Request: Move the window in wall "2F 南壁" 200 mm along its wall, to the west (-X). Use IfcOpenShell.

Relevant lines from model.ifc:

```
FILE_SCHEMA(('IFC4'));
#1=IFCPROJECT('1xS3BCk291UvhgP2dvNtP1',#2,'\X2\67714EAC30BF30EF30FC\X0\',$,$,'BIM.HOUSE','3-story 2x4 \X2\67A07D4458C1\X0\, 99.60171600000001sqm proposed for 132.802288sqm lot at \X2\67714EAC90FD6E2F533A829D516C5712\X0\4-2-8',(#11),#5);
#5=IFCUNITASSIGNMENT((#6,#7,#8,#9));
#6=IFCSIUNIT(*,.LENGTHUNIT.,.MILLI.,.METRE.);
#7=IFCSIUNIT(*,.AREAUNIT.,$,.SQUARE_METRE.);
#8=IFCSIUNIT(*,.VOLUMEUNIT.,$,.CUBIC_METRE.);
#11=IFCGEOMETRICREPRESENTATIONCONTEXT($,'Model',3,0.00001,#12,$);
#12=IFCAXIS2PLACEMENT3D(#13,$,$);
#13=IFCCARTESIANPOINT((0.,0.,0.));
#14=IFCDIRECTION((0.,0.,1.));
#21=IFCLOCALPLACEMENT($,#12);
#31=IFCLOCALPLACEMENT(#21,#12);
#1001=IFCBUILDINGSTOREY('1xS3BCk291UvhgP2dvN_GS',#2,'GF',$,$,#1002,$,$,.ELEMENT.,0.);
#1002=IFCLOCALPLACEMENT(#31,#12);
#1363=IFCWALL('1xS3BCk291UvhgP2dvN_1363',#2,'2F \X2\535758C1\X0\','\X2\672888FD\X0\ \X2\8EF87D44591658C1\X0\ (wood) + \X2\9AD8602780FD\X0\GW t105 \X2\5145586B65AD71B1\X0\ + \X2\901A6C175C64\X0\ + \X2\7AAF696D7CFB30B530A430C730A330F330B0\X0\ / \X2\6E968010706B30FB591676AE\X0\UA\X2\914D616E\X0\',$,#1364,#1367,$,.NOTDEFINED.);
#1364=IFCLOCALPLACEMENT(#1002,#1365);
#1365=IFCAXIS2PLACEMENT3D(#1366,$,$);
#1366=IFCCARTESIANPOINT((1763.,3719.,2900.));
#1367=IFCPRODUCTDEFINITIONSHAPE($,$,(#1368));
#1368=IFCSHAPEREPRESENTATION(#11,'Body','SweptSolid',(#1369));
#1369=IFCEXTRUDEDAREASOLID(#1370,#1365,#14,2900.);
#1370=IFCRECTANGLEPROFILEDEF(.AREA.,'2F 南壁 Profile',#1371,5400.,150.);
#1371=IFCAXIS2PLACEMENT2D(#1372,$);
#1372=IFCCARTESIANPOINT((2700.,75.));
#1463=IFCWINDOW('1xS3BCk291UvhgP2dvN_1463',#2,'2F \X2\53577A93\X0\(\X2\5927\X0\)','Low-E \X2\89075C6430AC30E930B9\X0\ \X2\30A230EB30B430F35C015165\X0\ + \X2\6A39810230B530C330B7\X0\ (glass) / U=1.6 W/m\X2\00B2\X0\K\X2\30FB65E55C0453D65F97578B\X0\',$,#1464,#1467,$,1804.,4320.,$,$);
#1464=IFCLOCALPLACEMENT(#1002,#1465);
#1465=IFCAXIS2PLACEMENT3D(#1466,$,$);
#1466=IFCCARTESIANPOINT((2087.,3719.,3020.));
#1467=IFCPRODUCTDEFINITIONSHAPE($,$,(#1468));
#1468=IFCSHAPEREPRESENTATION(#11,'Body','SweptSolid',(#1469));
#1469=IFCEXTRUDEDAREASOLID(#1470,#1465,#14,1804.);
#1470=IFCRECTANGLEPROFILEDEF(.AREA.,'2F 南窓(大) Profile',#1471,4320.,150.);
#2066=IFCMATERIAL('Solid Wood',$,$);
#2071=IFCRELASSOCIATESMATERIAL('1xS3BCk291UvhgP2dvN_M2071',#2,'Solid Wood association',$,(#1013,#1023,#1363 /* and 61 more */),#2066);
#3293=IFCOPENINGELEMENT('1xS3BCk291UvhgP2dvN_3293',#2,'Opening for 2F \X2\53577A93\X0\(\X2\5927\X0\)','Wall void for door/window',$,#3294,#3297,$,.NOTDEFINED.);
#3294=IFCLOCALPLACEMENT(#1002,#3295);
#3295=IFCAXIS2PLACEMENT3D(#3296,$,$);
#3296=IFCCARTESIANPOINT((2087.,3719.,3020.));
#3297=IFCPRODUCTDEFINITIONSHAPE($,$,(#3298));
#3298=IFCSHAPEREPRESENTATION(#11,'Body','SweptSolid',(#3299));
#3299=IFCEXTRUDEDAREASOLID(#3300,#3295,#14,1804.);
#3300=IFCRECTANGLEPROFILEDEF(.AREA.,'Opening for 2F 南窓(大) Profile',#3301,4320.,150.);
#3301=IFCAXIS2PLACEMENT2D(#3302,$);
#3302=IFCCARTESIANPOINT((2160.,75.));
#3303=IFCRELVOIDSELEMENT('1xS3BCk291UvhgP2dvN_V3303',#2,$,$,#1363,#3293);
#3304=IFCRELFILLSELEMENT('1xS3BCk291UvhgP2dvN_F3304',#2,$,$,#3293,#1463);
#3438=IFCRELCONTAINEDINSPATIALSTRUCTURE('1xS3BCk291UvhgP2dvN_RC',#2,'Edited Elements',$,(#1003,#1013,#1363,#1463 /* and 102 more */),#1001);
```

```python
import ifcopenshell
import ifcopenshell.api.geometry
import ifcopenshell.util.placement

model = ifcopenshell.open("model.ifc")

window = model.by_guid("1xS3BCk291UvhgP2dvN_1463")
opening = window.FillsVoids[0].RelatingOpeningElement
wall = opening.VoidsElements[0].RelatingBuildingElement

wall_matrix = ifcopenshell.util.placement.get_local_placement(wall.ObjectPlacement)
shift = wall_matrix[:3, 0] * -200.0
before = ifcopenshell.util.placement.get_local_placement(window.ObjectPlacement)[:3, 3].copy()

# The window is not placed relative to its opening, so move both.
for product in (opening, window):
    matrix = ifcopenshell.util.placement.get_local_placement(product.ObjectPlacement)
    matrix[:3, 3] += shift
    ifcopenshell.api.geometry.edit_object_placement(model, product=product, matrix=matrix, is_si=False)

after = ifcopenshell.util.placement.get_local_placement(window.ObjectPlacement)[:3, 3]
print("window moved by", (after - before).round(3) + 0.0)

model.write("model_v2.ifc")
```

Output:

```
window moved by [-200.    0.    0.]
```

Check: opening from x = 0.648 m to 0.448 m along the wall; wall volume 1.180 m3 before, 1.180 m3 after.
